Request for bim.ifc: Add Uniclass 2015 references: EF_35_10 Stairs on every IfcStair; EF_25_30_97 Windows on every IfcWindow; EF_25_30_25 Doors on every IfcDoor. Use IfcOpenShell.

First a look at what the model holds.

```python
import ifcopenshell

model = ifcopenshell.open("bim.ifc")
print(model.schema)
print("classifications:", [c.Name for c in model.by_type("IfcClassification")])
for ifc_class in ("IfcDoor", "IfcRoof", "IfcStair", "IfcWall", "IfcWindow"):
    print(ifc_class, len(model.by_type(ifc_class)))
```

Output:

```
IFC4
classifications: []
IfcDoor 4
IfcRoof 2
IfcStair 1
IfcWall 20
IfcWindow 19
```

```python
import ifcopenshell
import ifcopenshell.api.classification

model = ifcopenshell.open("bim.ifc")

system = ifcopenshell.api.classification.add_classification(model, classification="Uniclass 2015")

codes = {
    "IfcStair": ("EF_35_10", "Stairs"),
    "IfcWindow": ("EF_25_30_97", "Windows"),
    "IfcDoor": ("EF_25_30_25", "Doors"),
}
for ifc_class, (code, name) in codes.items():
    products = model.by_type(ifc_class)
    ifcopenshell.api.classification.add_reference(
        model, products=products, classification=system, identification=code, name=name
    )
    print(code, len(products))

model.write("bim-out.ifc")
```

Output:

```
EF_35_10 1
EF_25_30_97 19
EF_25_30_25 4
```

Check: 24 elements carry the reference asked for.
